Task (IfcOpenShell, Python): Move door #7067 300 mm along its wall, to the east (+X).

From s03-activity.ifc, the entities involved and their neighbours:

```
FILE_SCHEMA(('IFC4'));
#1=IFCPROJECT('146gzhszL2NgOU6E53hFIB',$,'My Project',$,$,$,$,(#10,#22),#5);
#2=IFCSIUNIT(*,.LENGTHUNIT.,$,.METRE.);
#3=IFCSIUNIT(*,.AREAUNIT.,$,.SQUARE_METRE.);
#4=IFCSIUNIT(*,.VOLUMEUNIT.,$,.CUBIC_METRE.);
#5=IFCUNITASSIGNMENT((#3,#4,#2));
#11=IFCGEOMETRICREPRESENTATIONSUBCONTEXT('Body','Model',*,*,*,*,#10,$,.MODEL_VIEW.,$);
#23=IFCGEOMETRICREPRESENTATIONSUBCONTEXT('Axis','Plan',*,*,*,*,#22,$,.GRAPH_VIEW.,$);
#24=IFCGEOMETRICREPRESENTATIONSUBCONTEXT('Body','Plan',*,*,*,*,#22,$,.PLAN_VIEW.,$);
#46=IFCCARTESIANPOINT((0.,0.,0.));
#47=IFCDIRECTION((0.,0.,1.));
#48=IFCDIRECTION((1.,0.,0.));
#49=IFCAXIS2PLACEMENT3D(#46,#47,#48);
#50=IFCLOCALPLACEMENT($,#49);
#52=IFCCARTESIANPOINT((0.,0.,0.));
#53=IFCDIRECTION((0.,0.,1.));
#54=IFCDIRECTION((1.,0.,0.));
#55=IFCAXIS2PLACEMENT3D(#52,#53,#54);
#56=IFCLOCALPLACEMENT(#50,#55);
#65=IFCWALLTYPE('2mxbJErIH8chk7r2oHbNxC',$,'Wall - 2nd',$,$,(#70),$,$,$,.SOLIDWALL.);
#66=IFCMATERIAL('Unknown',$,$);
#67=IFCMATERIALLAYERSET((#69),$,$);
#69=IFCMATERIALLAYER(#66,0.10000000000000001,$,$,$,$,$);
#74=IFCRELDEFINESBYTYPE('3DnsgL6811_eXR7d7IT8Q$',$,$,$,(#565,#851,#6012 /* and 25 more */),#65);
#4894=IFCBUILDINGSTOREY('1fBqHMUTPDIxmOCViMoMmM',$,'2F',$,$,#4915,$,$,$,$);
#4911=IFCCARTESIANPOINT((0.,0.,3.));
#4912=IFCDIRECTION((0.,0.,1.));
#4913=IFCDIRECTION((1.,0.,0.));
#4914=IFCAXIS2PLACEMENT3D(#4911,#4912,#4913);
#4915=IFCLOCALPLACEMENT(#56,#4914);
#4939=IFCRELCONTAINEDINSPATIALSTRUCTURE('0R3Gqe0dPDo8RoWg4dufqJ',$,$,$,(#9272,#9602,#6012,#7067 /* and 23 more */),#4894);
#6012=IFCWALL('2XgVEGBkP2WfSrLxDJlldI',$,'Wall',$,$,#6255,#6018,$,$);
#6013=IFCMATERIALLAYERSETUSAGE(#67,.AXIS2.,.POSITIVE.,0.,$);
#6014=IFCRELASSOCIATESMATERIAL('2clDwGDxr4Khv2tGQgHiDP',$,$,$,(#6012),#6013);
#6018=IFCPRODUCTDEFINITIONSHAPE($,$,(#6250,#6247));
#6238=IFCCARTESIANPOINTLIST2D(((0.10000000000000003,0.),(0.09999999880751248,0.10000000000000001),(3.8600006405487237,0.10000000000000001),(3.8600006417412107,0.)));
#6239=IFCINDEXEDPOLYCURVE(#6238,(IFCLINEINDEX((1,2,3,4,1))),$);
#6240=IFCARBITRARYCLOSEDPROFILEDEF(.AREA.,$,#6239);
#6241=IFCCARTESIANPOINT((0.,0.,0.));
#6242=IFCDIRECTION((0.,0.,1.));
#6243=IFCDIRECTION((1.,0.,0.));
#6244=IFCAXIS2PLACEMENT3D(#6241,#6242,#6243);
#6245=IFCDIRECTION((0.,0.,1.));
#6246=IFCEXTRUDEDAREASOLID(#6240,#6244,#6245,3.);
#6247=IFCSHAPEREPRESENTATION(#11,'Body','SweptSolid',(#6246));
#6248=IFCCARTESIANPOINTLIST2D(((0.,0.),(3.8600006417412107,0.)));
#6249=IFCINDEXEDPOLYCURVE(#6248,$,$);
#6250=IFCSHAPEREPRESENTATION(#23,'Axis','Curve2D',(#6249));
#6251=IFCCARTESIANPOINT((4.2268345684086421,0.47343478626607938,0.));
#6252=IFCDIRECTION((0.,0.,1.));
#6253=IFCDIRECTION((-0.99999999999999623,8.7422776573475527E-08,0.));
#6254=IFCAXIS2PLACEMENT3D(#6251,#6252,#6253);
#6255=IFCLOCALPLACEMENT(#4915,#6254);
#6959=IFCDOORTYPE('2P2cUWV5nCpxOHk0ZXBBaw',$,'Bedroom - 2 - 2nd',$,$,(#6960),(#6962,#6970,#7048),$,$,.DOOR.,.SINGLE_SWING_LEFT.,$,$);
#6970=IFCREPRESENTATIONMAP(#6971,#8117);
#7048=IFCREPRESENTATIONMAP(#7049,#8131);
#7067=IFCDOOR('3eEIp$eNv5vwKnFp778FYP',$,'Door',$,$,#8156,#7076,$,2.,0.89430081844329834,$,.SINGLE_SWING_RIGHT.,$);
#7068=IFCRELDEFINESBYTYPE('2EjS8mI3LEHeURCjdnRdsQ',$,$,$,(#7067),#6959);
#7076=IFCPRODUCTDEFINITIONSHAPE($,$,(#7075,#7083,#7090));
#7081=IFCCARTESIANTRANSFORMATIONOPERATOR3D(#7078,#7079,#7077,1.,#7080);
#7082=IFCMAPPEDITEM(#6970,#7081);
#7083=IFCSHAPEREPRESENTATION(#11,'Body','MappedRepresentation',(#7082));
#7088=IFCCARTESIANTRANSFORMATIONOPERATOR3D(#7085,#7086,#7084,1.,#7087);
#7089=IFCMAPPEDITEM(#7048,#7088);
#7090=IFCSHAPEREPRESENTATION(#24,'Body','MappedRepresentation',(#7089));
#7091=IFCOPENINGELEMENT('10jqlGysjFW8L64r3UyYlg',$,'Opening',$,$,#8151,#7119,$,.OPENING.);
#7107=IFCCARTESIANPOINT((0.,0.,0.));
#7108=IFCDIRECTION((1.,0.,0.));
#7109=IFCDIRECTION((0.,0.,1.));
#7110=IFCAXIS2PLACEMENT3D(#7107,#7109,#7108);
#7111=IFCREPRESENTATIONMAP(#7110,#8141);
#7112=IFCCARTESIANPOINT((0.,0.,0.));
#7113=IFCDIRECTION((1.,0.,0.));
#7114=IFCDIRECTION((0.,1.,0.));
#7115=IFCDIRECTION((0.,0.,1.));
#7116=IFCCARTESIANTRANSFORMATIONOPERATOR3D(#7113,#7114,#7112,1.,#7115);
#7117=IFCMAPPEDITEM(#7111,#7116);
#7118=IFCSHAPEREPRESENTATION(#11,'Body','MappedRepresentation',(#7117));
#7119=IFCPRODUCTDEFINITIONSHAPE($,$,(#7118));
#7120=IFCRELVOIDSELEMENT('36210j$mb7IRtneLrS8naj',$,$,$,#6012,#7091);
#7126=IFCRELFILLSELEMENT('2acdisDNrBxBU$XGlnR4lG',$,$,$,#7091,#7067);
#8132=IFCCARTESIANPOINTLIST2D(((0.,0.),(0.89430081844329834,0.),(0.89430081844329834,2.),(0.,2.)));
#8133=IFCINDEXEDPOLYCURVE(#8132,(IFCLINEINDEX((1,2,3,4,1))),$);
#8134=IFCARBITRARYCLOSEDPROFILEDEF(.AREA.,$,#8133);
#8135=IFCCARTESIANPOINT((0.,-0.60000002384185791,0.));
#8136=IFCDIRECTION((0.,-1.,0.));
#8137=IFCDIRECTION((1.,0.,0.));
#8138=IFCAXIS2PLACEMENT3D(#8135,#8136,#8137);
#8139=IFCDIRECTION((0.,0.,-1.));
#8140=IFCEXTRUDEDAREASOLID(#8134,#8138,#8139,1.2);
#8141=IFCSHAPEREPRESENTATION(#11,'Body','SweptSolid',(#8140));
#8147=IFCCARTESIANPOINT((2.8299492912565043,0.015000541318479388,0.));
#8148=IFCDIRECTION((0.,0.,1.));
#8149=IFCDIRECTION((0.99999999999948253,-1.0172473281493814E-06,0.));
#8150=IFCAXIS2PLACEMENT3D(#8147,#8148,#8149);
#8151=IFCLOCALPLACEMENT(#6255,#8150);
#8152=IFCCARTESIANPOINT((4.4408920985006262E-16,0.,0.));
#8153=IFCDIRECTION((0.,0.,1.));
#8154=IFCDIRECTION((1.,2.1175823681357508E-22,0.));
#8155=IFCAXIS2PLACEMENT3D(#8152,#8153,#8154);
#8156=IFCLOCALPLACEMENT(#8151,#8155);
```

```python
import ifcopenshell
import ifcopenshell.api.geometry
import ifcopenshell.util.placement
import ifcopenshell.util.unit

model = ifcopenshell.open("s03-activity.ifc")
unit_scale = ifcopenshell.util.unit.calculate_unit_scale(model)

door = model.by_id(7067)
opening = door.FillsVoids[0].RelatingOpeningElement
wall = opening.VoidsElements[0].RelatingBuildingElement

wall_matrix = ifcopenshell.util.placement.get_local_placement(wall.ObjectPlacement)
shift = wall_matrix[:3, 0] * -0.3 / unit_scale
before = ifcopenshell.util.placement.get_local_placement(door.ObjectPlacement)[:3, 3].copy()

# The door is placed relative to its opening, so it follows when the opening moves.
matrix = ifcopenshell.util.placement.get_local_placement(opening.ObjectPlacement)
matrix[:3, 3] += shift
ifcopenshell.api.geometry.edit_object_placement(
    model, product=opening, matrix=matrix, is_si=False, should_transform_children=True
)

after = ifcopenshell.util.placement.get_local_placement(door.ObjectPlacement)[:3, 3]
print("door moved by", (after - before).round(3) + 0.0)

model.write("s03-activity-out.ifc")
```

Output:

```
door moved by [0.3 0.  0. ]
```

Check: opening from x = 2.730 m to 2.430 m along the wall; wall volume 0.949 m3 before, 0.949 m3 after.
